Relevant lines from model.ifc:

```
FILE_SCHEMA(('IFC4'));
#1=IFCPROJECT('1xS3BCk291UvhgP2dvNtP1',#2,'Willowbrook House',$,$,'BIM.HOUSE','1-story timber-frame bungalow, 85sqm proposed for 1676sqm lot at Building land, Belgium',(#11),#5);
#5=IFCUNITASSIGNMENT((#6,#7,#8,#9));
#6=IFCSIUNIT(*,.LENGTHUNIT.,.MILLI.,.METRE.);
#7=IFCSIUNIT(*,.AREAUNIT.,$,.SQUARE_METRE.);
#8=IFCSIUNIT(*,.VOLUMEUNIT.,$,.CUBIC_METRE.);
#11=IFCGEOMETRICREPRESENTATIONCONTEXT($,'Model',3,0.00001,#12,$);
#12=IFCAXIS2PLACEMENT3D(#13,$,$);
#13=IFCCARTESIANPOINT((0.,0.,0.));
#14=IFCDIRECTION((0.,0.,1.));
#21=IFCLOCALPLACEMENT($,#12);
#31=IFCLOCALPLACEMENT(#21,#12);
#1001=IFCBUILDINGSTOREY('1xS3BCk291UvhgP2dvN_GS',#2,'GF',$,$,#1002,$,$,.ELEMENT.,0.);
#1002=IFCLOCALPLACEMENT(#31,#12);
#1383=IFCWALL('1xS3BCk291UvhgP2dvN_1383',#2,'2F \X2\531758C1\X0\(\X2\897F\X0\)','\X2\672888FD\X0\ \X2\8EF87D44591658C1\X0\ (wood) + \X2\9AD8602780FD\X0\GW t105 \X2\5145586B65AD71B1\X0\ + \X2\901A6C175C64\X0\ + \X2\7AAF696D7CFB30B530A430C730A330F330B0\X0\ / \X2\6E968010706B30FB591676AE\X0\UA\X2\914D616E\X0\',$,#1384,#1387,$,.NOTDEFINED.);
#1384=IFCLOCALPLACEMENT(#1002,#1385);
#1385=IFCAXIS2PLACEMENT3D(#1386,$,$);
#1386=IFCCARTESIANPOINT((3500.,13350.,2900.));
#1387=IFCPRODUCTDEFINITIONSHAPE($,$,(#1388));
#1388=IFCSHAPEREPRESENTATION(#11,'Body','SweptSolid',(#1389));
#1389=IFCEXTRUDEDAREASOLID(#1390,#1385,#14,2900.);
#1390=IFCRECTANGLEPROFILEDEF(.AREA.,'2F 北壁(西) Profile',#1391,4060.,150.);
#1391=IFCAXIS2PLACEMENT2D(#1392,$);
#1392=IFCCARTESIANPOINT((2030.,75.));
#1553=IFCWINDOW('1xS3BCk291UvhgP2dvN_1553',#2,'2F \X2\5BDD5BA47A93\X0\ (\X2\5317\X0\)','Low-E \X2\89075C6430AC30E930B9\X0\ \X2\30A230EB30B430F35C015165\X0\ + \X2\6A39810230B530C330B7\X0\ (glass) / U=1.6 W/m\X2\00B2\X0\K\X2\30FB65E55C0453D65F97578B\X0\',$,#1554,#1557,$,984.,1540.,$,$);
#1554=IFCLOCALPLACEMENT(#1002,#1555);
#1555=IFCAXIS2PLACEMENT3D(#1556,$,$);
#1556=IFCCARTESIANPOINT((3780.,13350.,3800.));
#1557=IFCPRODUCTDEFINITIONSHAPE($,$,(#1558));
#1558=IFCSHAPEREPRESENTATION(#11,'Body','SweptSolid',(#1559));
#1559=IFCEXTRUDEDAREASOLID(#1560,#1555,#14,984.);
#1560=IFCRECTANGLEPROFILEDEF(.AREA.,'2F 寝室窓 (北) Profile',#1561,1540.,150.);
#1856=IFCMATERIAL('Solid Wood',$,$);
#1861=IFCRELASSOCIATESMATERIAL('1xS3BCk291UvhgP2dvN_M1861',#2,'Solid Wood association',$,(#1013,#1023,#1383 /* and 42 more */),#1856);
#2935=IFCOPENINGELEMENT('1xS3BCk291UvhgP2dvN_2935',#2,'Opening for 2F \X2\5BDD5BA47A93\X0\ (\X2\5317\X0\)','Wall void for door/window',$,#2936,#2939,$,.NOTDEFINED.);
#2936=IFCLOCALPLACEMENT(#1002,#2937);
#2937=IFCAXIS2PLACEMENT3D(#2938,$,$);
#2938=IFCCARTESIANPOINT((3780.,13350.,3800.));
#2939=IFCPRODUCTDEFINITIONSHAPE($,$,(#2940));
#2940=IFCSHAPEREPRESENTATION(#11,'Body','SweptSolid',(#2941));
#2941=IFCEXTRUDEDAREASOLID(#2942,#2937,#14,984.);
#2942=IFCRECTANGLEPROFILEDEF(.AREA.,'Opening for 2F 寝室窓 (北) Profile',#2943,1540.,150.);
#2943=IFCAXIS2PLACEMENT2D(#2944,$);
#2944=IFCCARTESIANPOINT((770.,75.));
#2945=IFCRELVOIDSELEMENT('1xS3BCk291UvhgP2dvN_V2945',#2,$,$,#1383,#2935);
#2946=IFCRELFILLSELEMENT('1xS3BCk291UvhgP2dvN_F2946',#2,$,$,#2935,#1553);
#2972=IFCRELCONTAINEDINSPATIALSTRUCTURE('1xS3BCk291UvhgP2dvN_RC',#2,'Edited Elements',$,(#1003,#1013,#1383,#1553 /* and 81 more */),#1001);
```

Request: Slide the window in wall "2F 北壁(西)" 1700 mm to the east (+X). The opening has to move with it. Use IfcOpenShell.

```python
import ifcopenshell
import ifcopenshell.api.geometry
import ifcopenshell.util.placement

model = ifcopenshell.open("model.ifc")

window = model.by_id(1553)
opening = window.FillsVoids[0].RelatingOpeningElement
wall = opening.VoidsElements[0].RelatingBuildingElement

wall_matrix = ifcopenshell.util.placement.get_local_placement(wall.ObjectPlacement)
shift = wall_matrix[:3, 0] * 1700.0
before = ifcopenshell.util.placement.get_local_placement(window.ObjectPlacement)[:3, 3].copy()

# The window is not placed relative to its opening, so move both.
for product in (opening, window):
    matrix = ifcopenshell.util.placement.get_local_placement(product.ObjectPlacement)
    matrix[:3, 3] += shift
    ifcopenshell.api.geometry.edit_object_placement(model, product=product, matrix=matrix, is_si=False)

after = ifcopenshell.util.placement.get_local_placement(window.ObjectPlacement)[:3, 3]
print("window moved by", (after - before).round(3) + 0.0)

model.write("model_v2.ifc")
```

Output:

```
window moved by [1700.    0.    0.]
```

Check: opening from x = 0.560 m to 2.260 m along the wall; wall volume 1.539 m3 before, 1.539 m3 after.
